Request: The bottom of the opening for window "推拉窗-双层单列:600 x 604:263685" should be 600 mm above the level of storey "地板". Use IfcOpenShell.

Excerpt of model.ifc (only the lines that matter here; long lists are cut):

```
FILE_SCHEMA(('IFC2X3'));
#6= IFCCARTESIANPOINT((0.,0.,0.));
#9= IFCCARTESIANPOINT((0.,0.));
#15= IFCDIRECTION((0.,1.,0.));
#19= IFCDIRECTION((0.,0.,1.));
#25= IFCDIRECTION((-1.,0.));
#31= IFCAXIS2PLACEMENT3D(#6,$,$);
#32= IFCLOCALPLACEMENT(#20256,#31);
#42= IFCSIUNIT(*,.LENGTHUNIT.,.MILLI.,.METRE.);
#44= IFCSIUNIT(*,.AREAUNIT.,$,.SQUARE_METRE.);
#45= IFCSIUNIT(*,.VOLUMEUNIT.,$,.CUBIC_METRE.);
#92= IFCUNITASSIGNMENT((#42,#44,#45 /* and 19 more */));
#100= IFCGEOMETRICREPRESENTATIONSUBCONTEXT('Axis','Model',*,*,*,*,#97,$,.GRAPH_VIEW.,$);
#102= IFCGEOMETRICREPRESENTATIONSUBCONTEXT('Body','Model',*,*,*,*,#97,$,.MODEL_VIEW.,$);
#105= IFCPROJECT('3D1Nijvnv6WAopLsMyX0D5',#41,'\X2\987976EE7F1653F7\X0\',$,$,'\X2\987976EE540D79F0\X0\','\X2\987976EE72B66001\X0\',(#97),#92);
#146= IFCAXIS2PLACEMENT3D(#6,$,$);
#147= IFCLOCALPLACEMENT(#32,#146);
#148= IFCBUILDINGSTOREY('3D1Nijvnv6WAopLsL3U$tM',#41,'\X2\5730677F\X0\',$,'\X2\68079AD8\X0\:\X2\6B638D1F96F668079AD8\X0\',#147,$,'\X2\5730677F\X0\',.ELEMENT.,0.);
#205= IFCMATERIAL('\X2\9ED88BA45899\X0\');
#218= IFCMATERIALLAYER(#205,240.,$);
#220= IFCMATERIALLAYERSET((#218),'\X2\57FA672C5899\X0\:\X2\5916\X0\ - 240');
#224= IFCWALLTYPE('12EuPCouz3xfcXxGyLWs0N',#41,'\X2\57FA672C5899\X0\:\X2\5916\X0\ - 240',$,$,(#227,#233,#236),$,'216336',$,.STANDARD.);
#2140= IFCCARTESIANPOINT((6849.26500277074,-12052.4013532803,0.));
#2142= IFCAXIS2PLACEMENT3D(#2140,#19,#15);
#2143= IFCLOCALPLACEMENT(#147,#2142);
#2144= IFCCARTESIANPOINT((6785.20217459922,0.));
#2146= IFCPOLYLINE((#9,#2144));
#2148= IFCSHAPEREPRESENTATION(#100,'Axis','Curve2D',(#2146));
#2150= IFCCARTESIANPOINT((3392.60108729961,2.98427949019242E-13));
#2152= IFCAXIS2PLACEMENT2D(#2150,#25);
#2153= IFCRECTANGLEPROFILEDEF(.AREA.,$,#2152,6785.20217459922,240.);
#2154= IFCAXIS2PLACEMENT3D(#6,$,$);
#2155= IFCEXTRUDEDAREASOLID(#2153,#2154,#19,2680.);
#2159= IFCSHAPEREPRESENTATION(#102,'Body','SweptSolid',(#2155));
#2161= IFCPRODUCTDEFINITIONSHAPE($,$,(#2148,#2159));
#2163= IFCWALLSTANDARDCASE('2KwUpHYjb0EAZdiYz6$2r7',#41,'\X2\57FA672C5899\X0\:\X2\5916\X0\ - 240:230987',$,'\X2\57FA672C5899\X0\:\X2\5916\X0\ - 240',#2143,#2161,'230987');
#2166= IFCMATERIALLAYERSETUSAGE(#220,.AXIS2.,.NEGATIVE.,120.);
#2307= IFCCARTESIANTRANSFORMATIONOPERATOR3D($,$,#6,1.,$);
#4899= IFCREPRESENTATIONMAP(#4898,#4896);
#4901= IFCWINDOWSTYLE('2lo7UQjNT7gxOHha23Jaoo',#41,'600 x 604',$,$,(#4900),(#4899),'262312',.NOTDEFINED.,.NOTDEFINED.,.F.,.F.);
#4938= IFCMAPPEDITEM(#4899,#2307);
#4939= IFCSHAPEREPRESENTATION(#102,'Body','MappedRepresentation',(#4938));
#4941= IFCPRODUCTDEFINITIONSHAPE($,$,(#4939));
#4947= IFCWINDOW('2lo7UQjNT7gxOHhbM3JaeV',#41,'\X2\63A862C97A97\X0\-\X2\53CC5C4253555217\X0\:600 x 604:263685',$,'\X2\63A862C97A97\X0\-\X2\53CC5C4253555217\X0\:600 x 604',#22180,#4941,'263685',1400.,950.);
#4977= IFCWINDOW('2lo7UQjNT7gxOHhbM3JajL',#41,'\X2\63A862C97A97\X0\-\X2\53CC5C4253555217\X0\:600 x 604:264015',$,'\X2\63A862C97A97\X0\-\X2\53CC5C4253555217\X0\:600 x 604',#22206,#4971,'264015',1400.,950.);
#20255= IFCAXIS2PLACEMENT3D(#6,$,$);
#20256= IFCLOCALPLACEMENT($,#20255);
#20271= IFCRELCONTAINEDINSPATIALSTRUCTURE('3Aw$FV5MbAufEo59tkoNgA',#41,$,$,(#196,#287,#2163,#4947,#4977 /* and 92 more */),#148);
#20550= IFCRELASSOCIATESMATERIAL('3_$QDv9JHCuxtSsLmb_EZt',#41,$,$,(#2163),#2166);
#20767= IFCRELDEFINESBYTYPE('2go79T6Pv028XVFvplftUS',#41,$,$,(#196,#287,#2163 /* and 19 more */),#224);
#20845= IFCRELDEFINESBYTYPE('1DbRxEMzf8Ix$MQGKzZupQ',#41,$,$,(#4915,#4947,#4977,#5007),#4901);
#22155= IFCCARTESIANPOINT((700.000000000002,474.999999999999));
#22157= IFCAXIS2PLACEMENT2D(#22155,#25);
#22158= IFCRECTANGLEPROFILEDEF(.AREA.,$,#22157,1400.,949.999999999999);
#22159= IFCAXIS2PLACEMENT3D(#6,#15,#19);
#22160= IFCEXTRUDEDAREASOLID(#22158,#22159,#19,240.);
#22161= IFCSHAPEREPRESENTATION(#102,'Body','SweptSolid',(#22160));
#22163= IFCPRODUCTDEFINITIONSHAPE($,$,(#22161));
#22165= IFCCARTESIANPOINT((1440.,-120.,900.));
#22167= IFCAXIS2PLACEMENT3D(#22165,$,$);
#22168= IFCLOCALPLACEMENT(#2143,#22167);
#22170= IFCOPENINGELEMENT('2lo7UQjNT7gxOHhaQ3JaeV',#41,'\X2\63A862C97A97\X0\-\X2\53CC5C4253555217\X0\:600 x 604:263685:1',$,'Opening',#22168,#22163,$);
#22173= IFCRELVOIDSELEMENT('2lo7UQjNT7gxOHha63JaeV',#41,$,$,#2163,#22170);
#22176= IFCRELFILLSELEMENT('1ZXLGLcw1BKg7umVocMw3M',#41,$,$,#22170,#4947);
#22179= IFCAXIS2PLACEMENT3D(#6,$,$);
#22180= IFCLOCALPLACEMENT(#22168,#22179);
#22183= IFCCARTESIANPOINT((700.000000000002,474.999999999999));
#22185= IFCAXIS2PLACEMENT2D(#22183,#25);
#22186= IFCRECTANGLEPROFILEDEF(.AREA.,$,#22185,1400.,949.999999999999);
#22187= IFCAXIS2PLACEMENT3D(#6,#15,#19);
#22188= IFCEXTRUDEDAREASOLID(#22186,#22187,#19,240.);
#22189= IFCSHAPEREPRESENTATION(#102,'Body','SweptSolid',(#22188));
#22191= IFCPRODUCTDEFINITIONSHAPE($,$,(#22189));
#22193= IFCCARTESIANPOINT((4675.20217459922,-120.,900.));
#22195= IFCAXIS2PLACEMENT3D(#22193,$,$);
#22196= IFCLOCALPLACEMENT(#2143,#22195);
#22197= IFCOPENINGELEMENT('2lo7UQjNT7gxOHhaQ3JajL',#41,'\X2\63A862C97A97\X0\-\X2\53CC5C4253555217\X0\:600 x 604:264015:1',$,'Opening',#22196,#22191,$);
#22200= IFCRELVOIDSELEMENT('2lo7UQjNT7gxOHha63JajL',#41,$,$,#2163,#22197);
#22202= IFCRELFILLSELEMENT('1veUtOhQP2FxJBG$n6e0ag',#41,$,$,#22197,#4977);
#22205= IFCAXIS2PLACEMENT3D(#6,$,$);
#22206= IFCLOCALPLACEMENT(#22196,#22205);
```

```python
import numpy as np
import ifcopenshell
import ifcopenshell.api.geometry
import ifcopenshell.geom
import ifcopenshell.util.element
import ifcopenshell.util.placement
import ifcopenshell.util.shape
import ifcopenshell.util.unit

model = ifcopenshell.open("model.ifc")
unit_scale = ifcopenshell.util.unit.calculate_unit_scale(model)

window = model.by_id(4947)
opening = window.FillsVoids[0].RelatingOpeningElement
storey = ifcopenshell.util.element.get_container(window, ifc_class="IfcBuildingStorey")
level = ifcopenshell.util.placement.get_local_placement(storey.ObjectPlacement)[2, 3]

# The opening's origin need not be at the sill, so measure its lowest point.
shape = ifcopenshell.geom.create_shape(ifcopenshell.geom.settings(), opening)
bottom = ifcopenshell.util.shape.get_shape_bottom_elevation(shape, shape.geometry) / unit_scale
dz = level + 0.6 / unit_scale - bottom

shift = np.array([0.0, 0.0, dz])
# The window is placed relative to its opening, so it follows when the opening moves.
matrix = ifcopenshell.util.placement.get_local_placement(opening.ObjectPlacement)
matrix[:3, 3] += shift
ifcopenshell.api.geometry.edit_object_placement(
    model, product=opening, matrix=matrix, is_si=False, should_transform_children=True
)

print(f"moved by {dz * unit_scale:+.3f} m")

model.write("model_edited.ifc")
```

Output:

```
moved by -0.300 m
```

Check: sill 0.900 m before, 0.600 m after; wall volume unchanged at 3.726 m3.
